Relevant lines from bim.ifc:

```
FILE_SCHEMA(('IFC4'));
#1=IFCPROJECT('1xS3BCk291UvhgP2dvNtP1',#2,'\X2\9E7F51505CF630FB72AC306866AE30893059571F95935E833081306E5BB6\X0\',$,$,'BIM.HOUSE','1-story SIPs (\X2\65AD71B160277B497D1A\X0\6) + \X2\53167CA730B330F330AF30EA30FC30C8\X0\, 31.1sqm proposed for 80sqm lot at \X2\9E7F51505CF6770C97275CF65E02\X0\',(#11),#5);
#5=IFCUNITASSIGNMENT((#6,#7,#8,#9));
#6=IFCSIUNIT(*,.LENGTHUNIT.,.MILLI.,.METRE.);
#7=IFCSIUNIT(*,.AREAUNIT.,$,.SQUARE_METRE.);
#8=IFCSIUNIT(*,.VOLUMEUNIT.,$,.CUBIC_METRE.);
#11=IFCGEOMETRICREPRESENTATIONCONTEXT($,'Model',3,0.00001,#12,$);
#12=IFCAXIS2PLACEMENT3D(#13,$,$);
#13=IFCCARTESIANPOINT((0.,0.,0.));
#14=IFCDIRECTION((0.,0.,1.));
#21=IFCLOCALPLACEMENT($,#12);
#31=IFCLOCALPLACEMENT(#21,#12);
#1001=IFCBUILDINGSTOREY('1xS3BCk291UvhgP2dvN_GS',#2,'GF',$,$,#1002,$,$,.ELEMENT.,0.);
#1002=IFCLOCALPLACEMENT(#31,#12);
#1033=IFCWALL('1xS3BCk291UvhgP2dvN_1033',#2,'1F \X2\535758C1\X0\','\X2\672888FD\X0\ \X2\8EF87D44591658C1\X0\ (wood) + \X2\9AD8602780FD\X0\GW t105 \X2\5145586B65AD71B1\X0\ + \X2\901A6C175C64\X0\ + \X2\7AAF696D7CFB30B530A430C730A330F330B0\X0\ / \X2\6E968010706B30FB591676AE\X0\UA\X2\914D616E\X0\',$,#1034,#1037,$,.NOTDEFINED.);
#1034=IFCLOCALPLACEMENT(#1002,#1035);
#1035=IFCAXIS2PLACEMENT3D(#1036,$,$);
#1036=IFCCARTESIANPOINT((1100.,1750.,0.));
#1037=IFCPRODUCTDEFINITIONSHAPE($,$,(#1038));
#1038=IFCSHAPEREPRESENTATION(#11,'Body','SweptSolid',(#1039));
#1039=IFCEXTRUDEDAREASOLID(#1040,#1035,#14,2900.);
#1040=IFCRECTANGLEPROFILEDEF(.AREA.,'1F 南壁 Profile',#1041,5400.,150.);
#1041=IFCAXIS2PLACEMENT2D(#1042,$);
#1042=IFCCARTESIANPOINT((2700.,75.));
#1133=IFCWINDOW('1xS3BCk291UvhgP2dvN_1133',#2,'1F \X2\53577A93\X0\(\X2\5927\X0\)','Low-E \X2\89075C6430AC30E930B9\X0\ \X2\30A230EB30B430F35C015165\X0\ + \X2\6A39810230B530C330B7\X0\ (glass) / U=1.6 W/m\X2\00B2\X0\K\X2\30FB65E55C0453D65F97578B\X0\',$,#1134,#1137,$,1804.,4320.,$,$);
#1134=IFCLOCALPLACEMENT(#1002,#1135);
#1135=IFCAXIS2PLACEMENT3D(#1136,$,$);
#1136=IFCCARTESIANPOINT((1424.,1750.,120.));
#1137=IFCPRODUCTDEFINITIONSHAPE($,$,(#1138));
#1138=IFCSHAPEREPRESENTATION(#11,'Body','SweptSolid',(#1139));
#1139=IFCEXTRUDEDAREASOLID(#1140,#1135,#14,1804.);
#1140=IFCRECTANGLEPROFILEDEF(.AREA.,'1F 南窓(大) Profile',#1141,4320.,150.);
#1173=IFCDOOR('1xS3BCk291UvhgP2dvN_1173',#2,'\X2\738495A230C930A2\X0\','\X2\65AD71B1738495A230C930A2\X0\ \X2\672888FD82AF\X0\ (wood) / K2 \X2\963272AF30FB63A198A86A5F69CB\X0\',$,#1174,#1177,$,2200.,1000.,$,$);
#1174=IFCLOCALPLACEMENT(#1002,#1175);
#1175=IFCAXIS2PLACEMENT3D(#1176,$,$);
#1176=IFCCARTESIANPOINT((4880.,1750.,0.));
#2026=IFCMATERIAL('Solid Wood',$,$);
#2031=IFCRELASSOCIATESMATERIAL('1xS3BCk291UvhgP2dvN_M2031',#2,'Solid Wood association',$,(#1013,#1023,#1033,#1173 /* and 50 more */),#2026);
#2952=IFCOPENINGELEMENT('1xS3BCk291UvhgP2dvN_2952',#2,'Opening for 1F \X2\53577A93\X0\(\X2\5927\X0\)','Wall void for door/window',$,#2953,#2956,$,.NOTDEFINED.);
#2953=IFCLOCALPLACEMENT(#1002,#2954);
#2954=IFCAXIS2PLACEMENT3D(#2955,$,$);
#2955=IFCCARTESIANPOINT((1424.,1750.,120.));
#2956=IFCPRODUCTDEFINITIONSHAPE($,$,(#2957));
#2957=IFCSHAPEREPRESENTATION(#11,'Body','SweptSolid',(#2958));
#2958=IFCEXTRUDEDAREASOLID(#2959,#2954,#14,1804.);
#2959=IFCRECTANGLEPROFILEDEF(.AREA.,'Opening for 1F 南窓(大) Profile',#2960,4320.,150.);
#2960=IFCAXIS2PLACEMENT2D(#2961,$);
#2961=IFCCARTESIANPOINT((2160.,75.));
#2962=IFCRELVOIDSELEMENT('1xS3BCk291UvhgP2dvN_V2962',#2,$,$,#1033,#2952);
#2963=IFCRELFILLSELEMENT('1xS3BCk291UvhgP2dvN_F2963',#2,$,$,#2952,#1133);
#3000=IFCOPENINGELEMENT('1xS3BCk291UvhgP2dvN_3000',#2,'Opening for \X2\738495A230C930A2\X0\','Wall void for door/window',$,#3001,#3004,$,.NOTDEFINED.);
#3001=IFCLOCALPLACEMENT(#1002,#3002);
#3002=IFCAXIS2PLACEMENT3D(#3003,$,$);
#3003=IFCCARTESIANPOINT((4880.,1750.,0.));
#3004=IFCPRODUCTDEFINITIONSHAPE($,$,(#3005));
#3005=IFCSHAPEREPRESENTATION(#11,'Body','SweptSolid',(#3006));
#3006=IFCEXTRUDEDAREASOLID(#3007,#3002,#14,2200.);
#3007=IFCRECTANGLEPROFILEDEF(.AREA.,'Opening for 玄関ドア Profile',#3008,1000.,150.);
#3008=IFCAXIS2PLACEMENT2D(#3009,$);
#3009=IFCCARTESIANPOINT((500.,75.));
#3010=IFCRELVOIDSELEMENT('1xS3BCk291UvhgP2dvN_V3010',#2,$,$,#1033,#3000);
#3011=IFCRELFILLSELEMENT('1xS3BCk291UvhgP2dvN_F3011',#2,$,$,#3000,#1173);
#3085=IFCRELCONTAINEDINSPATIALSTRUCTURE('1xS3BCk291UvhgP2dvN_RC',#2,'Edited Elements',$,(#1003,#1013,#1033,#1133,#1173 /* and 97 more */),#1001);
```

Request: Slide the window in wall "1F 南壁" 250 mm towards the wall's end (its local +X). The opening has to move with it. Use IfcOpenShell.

```python
import ifcopenshell
import ifcopenshell.api.geometry
import ifcopenshell.util.placement
import ifcopenshell.util.unit

model = ifcopenshell.open("bim.ifc")
unit_scale = ifcopenshell.util.unit.calculate_unit_scale(model)

window = model.by_id(1133)
opening = window.FillsVoids[0].RelatingOpeningElement
wall = opening.VoidsElements[0].RelatingBuildingElement

wall_matrix = ifcopenshell.util.placement.get_local_placement(wall.ObjectPlacement)
shift = wall_matrix[:3, 0] * 0.25 / unit_scale
before = ifcopenshell.util.placement.get_local_placement(window.ObjectPlacement)[:3, 3].copy()

# The window is not placed relative to its opening, so move both.
for product in (opening, window):
    matrix = ifcopenshell.util.placement.get_local_placement(product.ObjectPlacement)
    matrix[:3, 3] += shift
    ifcopenshell.api.geometry.edit_object_placement(model, product=product, matrix=matrix, is_si=False)

after = ifcopenshell.util.placement.get_local_placement(window.ObjectPlacement)[:3, 3]
print("window moved by", (after - before).round(3) + 0.0)

model.write("bim_rev.ifc")
```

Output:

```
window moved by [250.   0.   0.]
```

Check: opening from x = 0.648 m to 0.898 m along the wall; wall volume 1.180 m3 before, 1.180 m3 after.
